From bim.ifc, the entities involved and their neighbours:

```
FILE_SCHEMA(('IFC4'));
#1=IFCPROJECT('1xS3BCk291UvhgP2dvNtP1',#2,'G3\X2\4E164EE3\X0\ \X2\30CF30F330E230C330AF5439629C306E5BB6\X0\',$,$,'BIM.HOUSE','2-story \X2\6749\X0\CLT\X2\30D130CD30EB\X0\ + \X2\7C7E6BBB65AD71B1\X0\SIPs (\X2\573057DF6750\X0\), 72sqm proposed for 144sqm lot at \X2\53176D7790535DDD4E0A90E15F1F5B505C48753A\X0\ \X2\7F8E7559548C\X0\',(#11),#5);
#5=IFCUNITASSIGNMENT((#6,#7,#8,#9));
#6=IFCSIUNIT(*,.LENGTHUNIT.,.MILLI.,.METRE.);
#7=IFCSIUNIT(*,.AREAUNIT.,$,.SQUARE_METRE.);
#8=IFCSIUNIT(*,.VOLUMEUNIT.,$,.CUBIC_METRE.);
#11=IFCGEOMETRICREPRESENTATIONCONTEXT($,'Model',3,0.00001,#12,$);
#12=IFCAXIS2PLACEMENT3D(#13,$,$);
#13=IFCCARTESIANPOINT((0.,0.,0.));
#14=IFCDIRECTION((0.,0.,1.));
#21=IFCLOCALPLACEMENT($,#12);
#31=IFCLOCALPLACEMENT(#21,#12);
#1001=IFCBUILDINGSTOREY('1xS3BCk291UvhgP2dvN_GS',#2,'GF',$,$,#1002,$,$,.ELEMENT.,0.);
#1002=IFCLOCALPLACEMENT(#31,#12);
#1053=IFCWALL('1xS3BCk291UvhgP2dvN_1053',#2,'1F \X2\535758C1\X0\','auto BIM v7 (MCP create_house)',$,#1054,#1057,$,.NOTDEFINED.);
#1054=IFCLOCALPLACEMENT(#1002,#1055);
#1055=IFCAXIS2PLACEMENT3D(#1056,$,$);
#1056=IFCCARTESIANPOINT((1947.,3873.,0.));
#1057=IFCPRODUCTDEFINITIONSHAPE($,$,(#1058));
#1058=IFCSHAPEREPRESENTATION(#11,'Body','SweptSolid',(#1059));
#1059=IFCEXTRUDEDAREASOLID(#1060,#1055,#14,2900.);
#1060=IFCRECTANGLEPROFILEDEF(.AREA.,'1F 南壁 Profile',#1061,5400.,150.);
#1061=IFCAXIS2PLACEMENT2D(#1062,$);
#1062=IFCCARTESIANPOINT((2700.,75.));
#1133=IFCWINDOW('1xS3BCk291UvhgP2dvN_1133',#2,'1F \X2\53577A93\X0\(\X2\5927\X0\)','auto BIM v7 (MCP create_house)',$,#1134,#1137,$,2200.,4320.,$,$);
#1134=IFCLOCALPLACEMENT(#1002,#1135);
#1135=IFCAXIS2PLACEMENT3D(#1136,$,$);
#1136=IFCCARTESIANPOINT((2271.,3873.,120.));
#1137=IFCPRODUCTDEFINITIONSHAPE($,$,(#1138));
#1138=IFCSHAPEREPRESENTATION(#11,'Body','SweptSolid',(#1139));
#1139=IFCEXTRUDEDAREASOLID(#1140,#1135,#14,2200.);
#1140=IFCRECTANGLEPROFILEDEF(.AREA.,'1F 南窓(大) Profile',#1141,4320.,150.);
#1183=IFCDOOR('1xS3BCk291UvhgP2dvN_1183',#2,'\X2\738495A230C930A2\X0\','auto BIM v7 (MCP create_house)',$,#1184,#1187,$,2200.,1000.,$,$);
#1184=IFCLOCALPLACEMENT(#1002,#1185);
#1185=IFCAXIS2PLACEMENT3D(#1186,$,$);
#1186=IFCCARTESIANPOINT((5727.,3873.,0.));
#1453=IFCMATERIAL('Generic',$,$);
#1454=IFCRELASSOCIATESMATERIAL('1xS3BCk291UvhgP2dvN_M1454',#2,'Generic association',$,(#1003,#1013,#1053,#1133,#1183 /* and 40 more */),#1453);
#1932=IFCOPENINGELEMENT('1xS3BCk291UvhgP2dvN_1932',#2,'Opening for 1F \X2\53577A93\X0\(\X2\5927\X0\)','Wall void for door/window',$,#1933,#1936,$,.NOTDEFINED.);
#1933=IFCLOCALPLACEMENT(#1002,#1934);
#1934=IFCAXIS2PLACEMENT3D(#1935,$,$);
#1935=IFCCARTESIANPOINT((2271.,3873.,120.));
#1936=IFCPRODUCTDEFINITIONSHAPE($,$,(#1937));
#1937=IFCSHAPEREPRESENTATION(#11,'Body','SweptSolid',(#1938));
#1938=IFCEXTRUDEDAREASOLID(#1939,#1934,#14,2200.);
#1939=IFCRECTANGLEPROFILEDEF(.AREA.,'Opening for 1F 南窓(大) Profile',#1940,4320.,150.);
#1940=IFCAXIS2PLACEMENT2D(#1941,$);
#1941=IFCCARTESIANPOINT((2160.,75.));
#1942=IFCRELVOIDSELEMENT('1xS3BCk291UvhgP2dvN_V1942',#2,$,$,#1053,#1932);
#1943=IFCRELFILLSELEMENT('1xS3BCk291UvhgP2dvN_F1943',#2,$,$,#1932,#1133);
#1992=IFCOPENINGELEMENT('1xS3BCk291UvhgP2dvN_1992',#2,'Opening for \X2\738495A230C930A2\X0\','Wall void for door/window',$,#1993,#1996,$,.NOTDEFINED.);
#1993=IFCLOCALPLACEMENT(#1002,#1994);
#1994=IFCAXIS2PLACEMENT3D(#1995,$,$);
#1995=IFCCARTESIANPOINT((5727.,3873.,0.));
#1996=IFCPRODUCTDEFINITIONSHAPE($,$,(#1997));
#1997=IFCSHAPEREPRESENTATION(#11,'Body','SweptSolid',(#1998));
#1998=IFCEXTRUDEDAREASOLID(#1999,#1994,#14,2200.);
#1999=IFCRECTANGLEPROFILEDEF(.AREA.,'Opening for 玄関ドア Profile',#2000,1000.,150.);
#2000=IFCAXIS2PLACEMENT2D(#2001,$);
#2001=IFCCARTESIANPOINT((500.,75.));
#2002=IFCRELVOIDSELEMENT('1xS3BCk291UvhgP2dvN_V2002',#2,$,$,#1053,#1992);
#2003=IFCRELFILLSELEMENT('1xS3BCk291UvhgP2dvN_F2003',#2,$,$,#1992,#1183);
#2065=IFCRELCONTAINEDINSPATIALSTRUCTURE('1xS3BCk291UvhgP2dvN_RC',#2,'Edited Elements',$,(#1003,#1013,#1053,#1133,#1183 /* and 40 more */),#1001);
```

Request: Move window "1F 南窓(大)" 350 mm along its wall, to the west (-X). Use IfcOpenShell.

```python
import ifcopenshell
import ifcopenshell.api.geometry
import ifcopenshell.util.placement
import ifcopenshell.util.unit

model = ifcopenshell.open("bim.ifc")
unit_scale = ifcopenshell.util.unit.calculate_unit_scale(model)

window = model.by_id(1133)
opening = window.FillsVoids[0].RelatingOpeningElement
wall = opening.VoidsElements[0].RelatingBuildingElement

wall_matrix = ifcopenshell.util.placement.get_local_placement(wall.ObjectPlacement)
shift = wall_matrix[:3, 0] * -0.35 / unit_scale
before = ifcopenshell.util.placement.get_local_placement(window.ObjectPlacement)[:3, 3].copy()

# The window is not placed relative to its opening, so move both.
for product in (opening, window):
    matrix = ifcopenshell.util.placement.get_local_placement(product.ObjectPlacement)
    matrix[:3, 3] += shift
    ifcopenshell.api.geometry.edit_object_placement(model, product=product, matrix=matrix, is_si=False)

after = ifcopenshell.util.placement.get_local_placement(window.ObjectPlacement)[:3, 3]
print("window moved by", (after - before).round(3) + 0.0)

model.write("bim_edited.ifc")
```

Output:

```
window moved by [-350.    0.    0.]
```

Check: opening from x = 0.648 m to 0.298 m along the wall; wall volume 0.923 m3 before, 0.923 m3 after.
